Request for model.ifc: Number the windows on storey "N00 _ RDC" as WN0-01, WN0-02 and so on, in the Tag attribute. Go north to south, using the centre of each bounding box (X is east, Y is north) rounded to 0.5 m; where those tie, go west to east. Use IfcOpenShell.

First a look at what the model holds.

```python
import ifcopenshell
import ifcopenshell.util.element
import ifcopenshell.util.placement

model = ifcopenshell.open("model.ifc")
print(model.schema)
storey = next(s for s in model.by_type("IfcBuildingStorey") if s.Name == "N00 _ RDC")
windows = [e for e in ifcopenshell.util.element.get_decomposition(storey) if e.is_a("IfcWindow")]
for e in sorted(windows, key=lambda e: e.id()):
    origin = ifcopenshell.util.placement.get_local_placement(e.ObjectPlacement)[:3, 3]
    print(e.id(), e.Tag, e.Name, origin.round(2) + 0.0, sep=" | ")
```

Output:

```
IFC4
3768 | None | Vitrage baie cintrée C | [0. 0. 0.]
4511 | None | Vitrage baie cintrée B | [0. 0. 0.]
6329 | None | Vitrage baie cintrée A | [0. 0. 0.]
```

```python
import ifcopenshell
import ifcopenshell.geom
import ifcopenshell.util.element
import ifcopenshell.util.shape

model = ifcopenshell.open("model.ifc")
settings = ifcopenshell.geom.settings()
settings.set("use-world-coords", True)


def centre(element):
    shape = ifcopenshell.geom.create_shape(settings, element)
    return ifcopenshell.util.shape.get_bbox_centroid(shape.geometry)


storey = next(s for s in model.by_type("IfcBuildingStorey") if s.Name == "N00 _ RDC")
windows = [e for e in ifcopenshell.util.element.get_decomposition(storey) if e.is_a("IfcWindow")]

# Insertion points can sit at a corner or the storey origin, so sort by the geometry (in metres).
centres = {e: centre(e) for e in windows}
windows.sort(key=lambda e: (-round(centres[e][1] / 0.5), centres[e][0]))

for i, e in enumerate(windows, start=1):
    number = f"WN0-{i:02d}"
    e.Tag = number
    print(e.id(), number)

model.write("model-out.ifc")
```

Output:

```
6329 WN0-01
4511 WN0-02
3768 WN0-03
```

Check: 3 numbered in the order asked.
